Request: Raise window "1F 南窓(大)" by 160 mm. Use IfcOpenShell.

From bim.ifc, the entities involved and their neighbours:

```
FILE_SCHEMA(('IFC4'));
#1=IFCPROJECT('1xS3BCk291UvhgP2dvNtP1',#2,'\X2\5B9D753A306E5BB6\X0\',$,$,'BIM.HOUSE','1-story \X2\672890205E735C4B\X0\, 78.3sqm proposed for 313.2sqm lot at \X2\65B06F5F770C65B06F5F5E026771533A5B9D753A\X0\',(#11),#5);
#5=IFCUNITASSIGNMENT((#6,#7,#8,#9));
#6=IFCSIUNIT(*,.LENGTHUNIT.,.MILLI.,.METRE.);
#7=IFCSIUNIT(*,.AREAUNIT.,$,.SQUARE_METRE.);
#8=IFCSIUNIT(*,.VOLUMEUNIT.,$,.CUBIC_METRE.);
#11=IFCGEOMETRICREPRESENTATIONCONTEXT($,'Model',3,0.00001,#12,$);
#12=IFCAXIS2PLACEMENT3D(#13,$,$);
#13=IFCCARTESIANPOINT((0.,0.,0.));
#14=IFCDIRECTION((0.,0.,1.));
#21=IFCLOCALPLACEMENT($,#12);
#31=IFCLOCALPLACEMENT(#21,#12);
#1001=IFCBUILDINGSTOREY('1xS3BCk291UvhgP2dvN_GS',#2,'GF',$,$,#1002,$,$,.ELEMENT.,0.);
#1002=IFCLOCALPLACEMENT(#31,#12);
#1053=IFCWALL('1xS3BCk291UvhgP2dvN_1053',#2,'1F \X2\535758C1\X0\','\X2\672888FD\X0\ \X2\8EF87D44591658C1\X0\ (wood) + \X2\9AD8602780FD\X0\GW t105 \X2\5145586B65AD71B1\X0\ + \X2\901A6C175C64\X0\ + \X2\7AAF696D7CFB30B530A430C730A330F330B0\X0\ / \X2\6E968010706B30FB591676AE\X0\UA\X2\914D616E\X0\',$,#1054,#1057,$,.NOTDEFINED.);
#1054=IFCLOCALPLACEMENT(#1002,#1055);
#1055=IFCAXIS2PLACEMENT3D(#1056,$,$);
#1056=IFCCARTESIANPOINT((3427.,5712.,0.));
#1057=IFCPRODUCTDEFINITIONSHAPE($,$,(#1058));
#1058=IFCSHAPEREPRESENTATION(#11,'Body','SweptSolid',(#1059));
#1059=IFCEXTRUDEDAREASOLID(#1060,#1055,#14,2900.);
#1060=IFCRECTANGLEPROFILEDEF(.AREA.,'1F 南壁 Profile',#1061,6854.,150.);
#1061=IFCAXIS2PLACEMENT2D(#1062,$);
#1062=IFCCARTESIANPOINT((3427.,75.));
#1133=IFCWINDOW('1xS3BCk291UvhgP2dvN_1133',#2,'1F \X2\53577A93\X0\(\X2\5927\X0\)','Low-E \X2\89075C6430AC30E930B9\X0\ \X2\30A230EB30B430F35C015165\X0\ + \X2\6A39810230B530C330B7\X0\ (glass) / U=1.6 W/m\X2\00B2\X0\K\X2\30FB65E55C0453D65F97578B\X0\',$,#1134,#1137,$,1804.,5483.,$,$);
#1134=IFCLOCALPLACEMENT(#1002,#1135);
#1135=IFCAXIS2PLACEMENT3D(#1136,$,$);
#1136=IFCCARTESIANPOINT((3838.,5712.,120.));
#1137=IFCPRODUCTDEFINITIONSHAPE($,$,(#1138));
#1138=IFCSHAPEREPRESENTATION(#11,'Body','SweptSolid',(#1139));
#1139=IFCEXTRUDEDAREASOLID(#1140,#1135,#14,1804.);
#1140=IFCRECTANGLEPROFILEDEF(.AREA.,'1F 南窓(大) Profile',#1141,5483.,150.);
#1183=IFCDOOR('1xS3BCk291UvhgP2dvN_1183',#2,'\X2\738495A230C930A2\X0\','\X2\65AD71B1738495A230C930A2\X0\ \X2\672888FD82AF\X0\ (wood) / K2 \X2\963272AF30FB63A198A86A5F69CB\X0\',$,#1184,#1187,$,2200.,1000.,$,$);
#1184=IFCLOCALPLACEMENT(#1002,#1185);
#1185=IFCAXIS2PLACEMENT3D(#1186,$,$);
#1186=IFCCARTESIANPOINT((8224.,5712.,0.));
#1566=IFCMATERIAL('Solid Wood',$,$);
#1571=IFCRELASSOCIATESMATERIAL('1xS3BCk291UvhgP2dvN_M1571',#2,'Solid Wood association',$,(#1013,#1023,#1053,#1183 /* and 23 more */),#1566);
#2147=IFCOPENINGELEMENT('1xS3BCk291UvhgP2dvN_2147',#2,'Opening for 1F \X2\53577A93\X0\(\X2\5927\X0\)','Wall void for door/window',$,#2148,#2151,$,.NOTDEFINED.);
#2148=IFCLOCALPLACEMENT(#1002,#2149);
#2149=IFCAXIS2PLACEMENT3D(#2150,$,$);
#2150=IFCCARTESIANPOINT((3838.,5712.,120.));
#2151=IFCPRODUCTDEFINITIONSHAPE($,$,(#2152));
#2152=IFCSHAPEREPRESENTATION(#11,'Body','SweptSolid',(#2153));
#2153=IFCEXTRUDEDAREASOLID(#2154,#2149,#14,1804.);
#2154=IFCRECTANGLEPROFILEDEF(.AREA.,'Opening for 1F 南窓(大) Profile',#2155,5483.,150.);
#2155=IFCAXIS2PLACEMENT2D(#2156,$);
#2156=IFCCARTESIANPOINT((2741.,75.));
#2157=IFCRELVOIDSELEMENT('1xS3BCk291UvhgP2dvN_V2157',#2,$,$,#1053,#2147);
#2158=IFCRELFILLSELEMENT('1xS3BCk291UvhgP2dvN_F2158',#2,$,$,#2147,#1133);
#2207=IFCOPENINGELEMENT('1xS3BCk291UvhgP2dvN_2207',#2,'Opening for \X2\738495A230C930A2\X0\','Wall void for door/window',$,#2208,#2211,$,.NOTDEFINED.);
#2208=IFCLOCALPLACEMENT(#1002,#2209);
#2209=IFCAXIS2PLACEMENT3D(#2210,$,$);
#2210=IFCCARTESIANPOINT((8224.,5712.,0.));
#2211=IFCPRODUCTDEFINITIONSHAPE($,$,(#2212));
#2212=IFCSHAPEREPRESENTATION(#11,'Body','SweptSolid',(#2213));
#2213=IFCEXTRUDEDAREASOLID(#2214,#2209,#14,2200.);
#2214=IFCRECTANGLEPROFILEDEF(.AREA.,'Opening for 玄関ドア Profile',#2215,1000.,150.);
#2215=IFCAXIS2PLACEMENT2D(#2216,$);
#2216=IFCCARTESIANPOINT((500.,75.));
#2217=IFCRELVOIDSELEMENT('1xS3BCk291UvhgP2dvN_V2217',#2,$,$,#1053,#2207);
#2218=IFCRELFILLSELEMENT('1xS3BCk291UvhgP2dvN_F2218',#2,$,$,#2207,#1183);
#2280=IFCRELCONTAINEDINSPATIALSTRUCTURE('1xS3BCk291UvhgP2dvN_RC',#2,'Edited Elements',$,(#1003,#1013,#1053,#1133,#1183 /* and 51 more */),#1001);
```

```python
import numpy as np
import ifcopenshell
import ifcopenshell.api.geometry
import ifcopenshell.util.placement
import ifcopenshell.util.unit

model = ifcopenshell.open("bim.ifc")
unit_scale = ifcopenshell.util.unit.calculate_unit_scale(model)

window = model.by_guid("1xS3BCk291UvhgP2dvN_1133")
opening = window.FillsVoids[0].RelatingOpeningElement
dz = 160.0

shift = np.array([0.0, 0.0, dz])
# The window is not placed relative to its opening, so move both.
for product in (opening, window):
    matrix = ifcopenshell.util.placement.get_local_placement(product.ObjectPlacement)
    matrix[:3, 3] += shift
    ifcopenshell.api.geometry.edit_object_placement(model, product=product, matrix=matrix, is_si=False)

print(f"moved by {dz * unit_scale:+.3f} m")

model.write("bim_v2.ifc")
```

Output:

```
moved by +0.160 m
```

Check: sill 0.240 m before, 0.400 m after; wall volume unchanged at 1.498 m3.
